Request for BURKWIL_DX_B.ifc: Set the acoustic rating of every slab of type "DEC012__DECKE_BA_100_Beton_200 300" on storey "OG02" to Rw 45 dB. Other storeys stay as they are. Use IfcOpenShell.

First a look at what the model holds.

```python
import ifcopenshell
import ifcopenshell.util.element

model = ifcopenshell.open("BURKWIL_DX_B.ifc")
print(model.schema)
storey = next(s for s in model.by_type("IfcBuildingStorey") if s.Name == "OG02")
slabs = [e for e in ifcopenshell.util.element.get_decomposition(storey) if e.is_a("IfcSlab")]
seen = {}
for e in slabs:
    element_type = ifcopenshell.util.element.get_type(e)
    key = (element_type.Name if element_type != e and element_type else None, ifcopenshell.util.element.get_pset(e, "Pset_SlabCommon", "AcousticRating"))
    seen[key] = seen.get(key, 0) + 1
for (name, value), count in sorted(seen.items(), key=str):
    print(count, "x", name, "|", value)
```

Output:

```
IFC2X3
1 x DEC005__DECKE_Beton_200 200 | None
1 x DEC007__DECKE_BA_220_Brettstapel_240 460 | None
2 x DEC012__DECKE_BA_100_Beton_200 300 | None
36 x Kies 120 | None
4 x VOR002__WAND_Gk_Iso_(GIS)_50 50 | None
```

```python
import ifcopenshell
import ifcopenshell.api.pset
import ifcopenshell.util.element

model = ifcopenshell.open("BURKWIL_DX_B.ifc")

storey = next(s for s in model.by_type("IfcBuildingStorey") if s.Name == "OG02")
slabs = [e for e in ifcopenshell.util.element.get_decomposition(storey) if e.is_a("IfcSlab")]

count = 0
for e in slabs:
    element_type = ifcopenshell.util.element.get_type(e)
    if element_type in (None, e) or element_type.Name != "DEC012__DECKE_BA_100_Beton_200 300":
        continue
    # add_pset returns the element's existing set when there is one.
    pset = ifcopenshell.api.pset.add_pset(model, product=e, name="Pset_SlabCommon")
    ifcopenshell.api.pset.edit_pset(model, pset=pset, properties={"AcousticRating": "Rw 45 dB"})
    count += 1

print(count, "slabs updated")

model.write("BURKWIL_DX_B_v2.ifc")
```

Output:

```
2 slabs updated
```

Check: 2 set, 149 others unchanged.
